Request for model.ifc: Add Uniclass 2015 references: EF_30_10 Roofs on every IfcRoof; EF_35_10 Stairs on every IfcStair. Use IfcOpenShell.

First a look at what the model holds.

```python
import ifcopenshell

model = ifcopenshell.open("model.ifc")
print(model.schema)
print("classifications:", [c.Name for c in model.by_type("IfcClassification")])
for ifc_class in ("IfcDoor", "IfcRoof", "IfcStair", "IfcWall", "IfcWindow"):
    print(ifc_class, len(model.by_type(ifc_class)))
```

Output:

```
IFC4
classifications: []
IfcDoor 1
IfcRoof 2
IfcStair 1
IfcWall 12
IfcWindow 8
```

```python
import ifcopenshell
import ifcopenshell.api.classification

model = ifcopenshell.open("model.ifc")

system = ifcopenshell.api.classification.add_classification(model, classification="Uniclass 2015")

codes = {
    "IfcRoof": ("EF_30_10", "Roofs"),
    "IfcStair": ("EF_35_10", "Stairs"),
}
for ifc_class, (code, name) in codes.items():
    products = model.by_type(ifc_class)
    ifcopenshell.api.classification.add_reference(
        model, products=products, classification=system, identification=code, name=name
    )
    print(code, len(products))

model.write("model_updated.ifc")
```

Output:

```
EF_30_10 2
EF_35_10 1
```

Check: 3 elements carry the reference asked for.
